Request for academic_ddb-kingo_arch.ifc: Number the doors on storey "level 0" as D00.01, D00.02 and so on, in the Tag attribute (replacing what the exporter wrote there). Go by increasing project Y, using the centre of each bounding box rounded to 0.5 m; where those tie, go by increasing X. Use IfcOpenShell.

First a look at what the model holds.

```python
import ifcopenshell
import ifcopenshell.util.element
import ifcopenshell.util.placement

model = ifcopenshell.open("academic_ddb-kingo_arch.ifc")
print(model.schema)
storey = next(s for s in model.by_type("IfcBuildingStorey") if s.Name == "level 0")
doors = [e for e in ifcopenshell.util.element.get_decomposition(storey) if e.is_a("IfcDoor")]
for e in sorted(doors, key=lambda e: e.id()):
    origin = ifcopenshell.util.placement.get_local_placement(e.ObjectPlacement)[:3, 3]
    print(e.id(), e.Tag, e.Name, origin.round(2) + 0.0, sep=" | ")
```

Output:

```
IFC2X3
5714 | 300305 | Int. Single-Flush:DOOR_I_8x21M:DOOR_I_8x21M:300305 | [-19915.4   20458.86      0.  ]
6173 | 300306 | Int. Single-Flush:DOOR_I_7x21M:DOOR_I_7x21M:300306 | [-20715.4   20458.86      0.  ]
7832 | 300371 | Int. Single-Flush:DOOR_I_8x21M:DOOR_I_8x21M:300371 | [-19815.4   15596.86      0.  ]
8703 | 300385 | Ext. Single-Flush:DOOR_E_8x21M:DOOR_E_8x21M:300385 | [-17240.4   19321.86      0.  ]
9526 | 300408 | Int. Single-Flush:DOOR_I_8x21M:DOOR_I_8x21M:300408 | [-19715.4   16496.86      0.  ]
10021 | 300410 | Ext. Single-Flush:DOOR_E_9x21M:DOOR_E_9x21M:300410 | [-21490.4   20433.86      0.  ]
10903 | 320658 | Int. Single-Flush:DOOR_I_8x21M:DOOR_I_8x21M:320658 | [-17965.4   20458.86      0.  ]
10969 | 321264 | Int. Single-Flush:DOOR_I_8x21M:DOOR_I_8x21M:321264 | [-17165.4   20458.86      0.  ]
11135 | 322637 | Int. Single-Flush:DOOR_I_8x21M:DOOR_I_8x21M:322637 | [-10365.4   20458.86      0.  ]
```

```python
import ifcopenshell
import ifcopenshell.geom
import ifcopenshell.util.element
import ifcopenshell.util.shape

model = ifcopenshell.open("academic_ddb-kingo_arch.ifc")
settings = ifcopenshell.geom.settings()
settings.set("use-world-coords", True)


def centre(element):
    shape = ifcopenshell.geom.create_shape(settings, element)
    return ifcopenshell.util.shape.get_bbox_centroid(shape.geometry)


storey = next(s for s in model.by_type("IfcBuildingStorey") if s.Name == "level 0")
doors = [e for e in ifcopenshell.util.element.get_decomposition(storey) if e.is_a("IfcDoor")]

# Insertion points can sit at a corner or the storey origin, so sort by the geometry (in metres).
centres = {e: centre(e) for e in doors}
doors.sort(key=lambda e: (round(centres[e][1] / 0.5), centres[e][0]))

for i, e in enumerate(doors, start=1):
    number = f"D00.{i:02d}"
    e.Tag = number
    print(e.id(), number)

model.write("academic_ddb-kingo_arch_rev.ifc")
```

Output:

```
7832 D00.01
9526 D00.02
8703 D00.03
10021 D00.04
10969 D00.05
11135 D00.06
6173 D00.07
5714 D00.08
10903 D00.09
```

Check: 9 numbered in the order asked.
